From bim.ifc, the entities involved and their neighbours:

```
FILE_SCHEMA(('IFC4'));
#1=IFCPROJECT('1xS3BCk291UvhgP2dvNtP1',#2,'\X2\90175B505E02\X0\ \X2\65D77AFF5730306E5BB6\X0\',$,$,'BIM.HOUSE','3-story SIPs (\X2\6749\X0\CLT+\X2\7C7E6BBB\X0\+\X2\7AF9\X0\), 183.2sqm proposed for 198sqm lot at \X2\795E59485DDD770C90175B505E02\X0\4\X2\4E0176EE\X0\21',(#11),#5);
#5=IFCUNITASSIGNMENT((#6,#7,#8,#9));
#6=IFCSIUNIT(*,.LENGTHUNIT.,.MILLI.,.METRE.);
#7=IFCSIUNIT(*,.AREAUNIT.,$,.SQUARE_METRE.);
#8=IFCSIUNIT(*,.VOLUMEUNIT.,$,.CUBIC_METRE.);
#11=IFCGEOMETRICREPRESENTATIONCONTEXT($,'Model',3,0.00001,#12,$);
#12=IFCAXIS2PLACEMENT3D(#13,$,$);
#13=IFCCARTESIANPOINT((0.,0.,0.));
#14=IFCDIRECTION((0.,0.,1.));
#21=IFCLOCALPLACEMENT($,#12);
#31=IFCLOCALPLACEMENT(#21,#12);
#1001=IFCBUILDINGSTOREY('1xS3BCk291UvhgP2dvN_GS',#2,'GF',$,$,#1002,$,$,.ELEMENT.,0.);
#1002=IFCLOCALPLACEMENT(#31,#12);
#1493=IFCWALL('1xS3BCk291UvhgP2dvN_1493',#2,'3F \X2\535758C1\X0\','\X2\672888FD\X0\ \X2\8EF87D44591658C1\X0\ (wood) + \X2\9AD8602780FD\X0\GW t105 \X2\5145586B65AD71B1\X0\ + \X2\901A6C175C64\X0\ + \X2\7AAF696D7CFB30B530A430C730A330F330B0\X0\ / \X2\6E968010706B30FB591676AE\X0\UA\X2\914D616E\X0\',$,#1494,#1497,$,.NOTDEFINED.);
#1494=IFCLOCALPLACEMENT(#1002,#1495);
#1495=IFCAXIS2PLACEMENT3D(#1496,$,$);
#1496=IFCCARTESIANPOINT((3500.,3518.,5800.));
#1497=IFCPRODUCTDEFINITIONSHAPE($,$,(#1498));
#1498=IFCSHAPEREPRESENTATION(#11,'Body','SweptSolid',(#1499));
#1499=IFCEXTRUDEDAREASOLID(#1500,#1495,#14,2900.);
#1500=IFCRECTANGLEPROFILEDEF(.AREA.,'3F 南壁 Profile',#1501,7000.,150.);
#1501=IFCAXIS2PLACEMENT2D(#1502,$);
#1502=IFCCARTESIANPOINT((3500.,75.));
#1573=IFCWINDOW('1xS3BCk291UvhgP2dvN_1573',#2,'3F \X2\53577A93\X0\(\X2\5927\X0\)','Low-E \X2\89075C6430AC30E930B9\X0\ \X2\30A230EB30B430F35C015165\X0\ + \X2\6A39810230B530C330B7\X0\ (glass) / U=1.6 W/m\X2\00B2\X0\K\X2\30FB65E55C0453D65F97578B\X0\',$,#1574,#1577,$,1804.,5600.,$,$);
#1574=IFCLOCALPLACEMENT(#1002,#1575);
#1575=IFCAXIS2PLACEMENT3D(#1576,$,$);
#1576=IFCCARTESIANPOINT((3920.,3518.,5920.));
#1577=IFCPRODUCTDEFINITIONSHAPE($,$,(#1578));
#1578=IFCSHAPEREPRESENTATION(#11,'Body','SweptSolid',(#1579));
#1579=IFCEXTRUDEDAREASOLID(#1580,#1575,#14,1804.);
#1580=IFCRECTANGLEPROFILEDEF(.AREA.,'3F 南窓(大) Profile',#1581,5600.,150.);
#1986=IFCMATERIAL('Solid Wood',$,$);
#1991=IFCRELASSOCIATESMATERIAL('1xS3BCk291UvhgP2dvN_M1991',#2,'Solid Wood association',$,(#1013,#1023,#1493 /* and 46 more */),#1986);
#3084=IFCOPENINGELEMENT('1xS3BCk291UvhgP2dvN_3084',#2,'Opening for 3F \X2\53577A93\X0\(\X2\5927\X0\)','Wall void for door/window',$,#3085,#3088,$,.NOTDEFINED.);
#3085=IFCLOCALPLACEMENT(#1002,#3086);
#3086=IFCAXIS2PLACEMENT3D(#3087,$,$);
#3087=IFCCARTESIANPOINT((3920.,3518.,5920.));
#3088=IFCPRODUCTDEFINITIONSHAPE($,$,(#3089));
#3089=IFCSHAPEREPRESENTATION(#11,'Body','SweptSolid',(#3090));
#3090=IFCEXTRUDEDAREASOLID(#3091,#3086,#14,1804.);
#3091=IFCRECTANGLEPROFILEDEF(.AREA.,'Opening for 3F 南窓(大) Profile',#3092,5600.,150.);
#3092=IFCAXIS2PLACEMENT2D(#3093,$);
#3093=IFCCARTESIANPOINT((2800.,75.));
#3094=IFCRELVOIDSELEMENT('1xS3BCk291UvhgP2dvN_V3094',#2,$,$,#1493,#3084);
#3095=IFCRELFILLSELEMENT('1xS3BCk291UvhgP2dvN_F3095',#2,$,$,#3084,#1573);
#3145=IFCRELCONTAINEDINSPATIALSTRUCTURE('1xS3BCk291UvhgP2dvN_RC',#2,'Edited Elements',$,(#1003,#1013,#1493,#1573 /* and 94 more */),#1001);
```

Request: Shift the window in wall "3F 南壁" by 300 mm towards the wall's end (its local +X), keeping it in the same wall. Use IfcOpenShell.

```python
import ifcopenshell
import ifcopenshell.api.geometry
import ifcopenshell.util.placement
import ifcopenshell.util.unit

model = ifcopenshell.open("bim.ifc")
unit_scale = ifcopenshell.util.unit.calculate_unit_scale(model)

window = model.by_guid("1xS3BCk291UvhgP2dvN_1573")
opening = window.FillsVoids[0].RelatingOpeningElement
wall = opening.VoidsElements[0].RelatingBuildingElement

wall_matrix = ifcopenshell.util.placement.get_local_placement(wall.ObjectPlacement)
shift = wall_matrix[:3, 0] * 0.3 / unit_scale
before = ifcopenshell.util.placement.get_local_placement(window.ObjectPlacement)[:3, 3].copy()

# The window is not placed relative to its opening, so move both.
for product in (opening, window):
    matrix = ifcopenshell.util.placement.get_local_placement(product.ObjectPlacement)
    matrix[:3, 3] += shift
    ifcopenshell.api.geometry.edit_object_placement(model, product=product, matrix=matrix, is_si=False)

after = ifcopenshell.util.placement.get_local_placement(window.ObjectPlacement)[:3, 3]
print("window moved by", (after - before).round(3) + 0.0)

model.write("bim_v2.ifc")
```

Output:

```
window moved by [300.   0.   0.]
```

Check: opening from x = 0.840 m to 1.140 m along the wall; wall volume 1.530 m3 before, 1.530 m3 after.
